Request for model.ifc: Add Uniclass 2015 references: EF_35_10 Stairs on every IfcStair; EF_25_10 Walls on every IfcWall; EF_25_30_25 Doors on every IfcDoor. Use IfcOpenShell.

First a look at what the model holds.

```python
import ifcopenshell

model = ifcopenshell.open("model.ifc")
print(model.schema)
print("classifications:", [c.Name for c in model.by_type("IfcClassification")])
for ifc_class in ("IfcDoor", "IfcRoof", "IfcStair", "IfcWall", "IfcWindow"):
    print(ifc_class, len(model.by_type(ifc_class)))
```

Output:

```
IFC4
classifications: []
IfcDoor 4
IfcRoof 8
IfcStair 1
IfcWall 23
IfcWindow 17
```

```python
import ifcopenshell
import ifcopenshell.api.classification

model = ifcopenshell.open("model.ifc")

system = ifcopenshell.api.classification.add_classification(model, classification="Uniclass 2015")

codes = {
    "IfcStair": ("EF_35_10", "Stairs"),
    "IfcWall": ("EF_25_10", "Walls"),
    "IfcDoor": ("EF_25_30_25", "Doors"),
}
for ifc_class, (code, name) in codes.items():
    products = model.by_type(ifc_class)
    ifcopenshell.api.classification.add_reference(
        model, products=products, classification=system, identification=code, name=name
    )
    print(code, len(products))

model.write("model_v2.ifc")
```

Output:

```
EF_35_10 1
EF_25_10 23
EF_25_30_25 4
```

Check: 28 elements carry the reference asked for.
